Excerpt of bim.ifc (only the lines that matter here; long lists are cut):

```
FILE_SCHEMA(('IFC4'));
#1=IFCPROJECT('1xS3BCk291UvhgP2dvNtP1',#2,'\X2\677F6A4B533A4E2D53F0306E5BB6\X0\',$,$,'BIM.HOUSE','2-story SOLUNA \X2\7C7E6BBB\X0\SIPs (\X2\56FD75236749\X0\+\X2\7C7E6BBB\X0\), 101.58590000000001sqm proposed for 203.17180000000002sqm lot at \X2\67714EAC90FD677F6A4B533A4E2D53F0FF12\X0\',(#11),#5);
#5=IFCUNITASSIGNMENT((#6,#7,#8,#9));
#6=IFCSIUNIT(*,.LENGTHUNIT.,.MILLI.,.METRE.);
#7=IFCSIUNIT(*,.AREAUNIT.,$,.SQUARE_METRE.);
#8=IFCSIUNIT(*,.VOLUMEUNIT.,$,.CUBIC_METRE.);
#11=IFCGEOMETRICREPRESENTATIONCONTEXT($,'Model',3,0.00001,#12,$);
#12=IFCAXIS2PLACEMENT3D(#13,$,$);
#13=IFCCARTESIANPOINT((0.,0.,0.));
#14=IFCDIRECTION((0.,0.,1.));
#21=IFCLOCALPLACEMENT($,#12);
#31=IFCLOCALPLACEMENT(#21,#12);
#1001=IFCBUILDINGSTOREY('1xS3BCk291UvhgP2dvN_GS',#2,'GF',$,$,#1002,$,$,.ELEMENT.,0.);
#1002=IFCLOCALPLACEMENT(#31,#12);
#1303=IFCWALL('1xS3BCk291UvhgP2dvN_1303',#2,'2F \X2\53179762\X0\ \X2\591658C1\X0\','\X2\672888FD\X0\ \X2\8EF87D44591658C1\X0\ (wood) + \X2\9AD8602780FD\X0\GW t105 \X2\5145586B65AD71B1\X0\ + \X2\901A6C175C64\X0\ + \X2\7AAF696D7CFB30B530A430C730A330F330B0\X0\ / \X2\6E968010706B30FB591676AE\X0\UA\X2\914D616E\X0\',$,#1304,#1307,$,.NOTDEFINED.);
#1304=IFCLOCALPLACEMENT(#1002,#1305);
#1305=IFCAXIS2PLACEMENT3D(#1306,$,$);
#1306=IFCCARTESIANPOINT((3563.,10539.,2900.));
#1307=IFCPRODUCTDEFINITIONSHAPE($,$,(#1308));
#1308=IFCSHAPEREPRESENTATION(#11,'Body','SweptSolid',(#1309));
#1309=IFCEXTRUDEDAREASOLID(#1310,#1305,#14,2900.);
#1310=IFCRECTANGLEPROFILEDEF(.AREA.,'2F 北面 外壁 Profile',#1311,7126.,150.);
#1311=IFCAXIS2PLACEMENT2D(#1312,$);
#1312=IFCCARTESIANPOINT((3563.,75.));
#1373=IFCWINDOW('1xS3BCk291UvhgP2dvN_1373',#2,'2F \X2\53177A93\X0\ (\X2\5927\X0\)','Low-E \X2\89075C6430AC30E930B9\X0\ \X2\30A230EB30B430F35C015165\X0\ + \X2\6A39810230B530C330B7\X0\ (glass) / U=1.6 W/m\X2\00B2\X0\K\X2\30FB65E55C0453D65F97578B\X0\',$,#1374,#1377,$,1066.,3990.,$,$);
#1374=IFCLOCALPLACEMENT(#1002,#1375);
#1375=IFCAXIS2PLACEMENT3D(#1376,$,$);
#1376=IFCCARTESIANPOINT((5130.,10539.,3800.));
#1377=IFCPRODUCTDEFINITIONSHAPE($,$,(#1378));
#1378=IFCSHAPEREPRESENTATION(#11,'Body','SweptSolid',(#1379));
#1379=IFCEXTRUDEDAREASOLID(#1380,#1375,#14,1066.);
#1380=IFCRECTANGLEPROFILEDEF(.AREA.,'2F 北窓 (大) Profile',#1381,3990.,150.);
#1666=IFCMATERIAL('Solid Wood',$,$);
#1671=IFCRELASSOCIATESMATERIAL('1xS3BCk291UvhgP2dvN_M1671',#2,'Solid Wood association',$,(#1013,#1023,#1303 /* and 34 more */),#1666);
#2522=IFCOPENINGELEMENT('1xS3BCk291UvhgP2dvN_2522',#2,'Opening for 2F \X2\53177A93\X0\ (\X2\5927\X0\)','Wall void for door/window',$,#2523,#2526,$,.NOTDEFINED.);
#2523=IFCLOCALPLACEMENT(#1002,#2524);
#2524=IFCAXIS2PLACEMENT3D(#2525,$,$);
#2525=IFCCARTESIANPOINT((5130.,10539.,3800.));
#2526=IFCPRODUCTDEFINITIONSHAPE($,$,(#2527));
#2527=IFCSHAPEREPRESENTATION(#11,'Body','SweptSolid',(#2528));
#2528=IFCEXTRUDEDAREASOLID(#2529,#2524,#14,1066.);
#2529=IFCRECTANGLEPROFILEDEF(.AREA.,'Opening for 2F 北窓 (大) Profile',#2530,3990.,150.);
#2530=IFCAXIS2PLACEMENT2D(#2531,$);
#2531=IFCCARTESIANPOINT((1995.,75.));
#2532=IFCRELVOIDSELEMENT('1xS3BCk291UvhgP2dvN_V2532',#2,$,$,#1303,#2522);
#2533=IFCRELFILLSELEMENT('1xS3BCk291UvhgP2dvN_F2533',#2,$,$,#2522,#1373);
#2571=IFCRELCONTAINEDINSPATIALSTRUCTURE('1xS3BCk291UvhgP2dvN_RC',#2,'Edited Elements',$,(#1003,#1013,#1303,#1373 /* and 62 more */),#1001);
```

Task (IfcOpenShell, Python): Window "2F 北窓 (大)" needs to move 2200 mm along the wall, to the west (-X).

```python
import ifcopenshell
import ifcopenshell.api.geometry
import ifcopenshell.util.placement

model = ifcopenshell.open("bim.ifc")

window = model.by_guid("1xS3BCk291UvhgP2dvN_1373")
opening = window.FillsVoids[0].RelatingOpeningElement
wall = opening.VoidsElements[0].RelatingBuildingElement

wall_matrix = ifcopenshell.util.placement.get_local_placement(wall.ObjectPlacement)
shift = wall_matrix[:3, 0] * -2200.0
before = ifcopenshell.util.placement.get_local_placement(window.ObjectPlacement)[:3, 3].copy()

# The window is not placed relative to its opening, so move both.
for product in (opening, window):
    matrix = ifcopenshell.util.placement.get_local_placement(product.ObjectPlacement)
    matrix[:3, 3] += shift
    ifcopenshell.api.geometry.edit_object_placement(model, product=product, matrix=matrix, is_si=False)

after = ifcopenshell.util.placement.get_local_placement(window.ObjectPlacement)[:3, 3]
print("window moved by", (after - before).round(3) + 0.0)

model.write("bim_updated.ifc")
```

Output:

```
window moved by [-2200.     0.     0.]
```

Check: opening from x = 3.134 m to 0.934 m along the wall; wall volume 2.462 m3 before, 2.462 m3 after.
